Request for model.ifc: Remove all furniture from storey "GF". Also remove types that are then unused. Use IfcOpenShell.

First a look at what the model holds.

```python
import ifcopenshell
import ifcopenshell.util.element

model = ifcopenshell.open("model.ifc")
print(model.schema)
storey = next(s for s in model.by_type("IfcBuildingStorey") if s.Name == "GF")
furniture = [e for e in ifcopenshell.util.element.get_decomposition(storey) if e.is_a("IfcFurnishingElement")]
seen = {}
for e in furniture:
    element_type = ifcopenshell.util.element.get_type(e)
    name = element_type.Name if element_type not in (None, e) else None
    seen[name] = seen.get(name, 0) + 1
for name, count in sorted(seen.items(), key=str):
    print(count, "x", name)
```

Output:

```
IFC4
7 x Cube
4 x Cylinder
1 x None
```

```python
import ifcopenshell
import ifcopenshell.api.root
import ifcopenshell.util.element

model = ifcopenshell.open("model.ifc")

storey = next(s for s in model.by_type("IfcBuildingStorey") if s.Name == "GF")
furniture = [e for e in ifcopenshell.util.element.get_decomposition(storey) if e.is_a("IfcFurnishingElement")]
types = {ifcopenshell.util.element.get_type(e) for e in furniture} - {None, *furniture}

for e in furniture:
    ifcopenshell.api.root.remove_product(model, product=e)
print(len(furniture), "removed")

unused = [t for t in types if not ifcopenshell.util.element.get_types(t)]
for t in unused:
    ifcopenshell.api.root.remove_product(model, product=t)
print(len(unused), "unused types removed")

model.write("model-out.ifc")
```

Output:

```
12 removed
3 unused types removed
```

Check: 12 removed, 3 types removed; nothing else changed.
